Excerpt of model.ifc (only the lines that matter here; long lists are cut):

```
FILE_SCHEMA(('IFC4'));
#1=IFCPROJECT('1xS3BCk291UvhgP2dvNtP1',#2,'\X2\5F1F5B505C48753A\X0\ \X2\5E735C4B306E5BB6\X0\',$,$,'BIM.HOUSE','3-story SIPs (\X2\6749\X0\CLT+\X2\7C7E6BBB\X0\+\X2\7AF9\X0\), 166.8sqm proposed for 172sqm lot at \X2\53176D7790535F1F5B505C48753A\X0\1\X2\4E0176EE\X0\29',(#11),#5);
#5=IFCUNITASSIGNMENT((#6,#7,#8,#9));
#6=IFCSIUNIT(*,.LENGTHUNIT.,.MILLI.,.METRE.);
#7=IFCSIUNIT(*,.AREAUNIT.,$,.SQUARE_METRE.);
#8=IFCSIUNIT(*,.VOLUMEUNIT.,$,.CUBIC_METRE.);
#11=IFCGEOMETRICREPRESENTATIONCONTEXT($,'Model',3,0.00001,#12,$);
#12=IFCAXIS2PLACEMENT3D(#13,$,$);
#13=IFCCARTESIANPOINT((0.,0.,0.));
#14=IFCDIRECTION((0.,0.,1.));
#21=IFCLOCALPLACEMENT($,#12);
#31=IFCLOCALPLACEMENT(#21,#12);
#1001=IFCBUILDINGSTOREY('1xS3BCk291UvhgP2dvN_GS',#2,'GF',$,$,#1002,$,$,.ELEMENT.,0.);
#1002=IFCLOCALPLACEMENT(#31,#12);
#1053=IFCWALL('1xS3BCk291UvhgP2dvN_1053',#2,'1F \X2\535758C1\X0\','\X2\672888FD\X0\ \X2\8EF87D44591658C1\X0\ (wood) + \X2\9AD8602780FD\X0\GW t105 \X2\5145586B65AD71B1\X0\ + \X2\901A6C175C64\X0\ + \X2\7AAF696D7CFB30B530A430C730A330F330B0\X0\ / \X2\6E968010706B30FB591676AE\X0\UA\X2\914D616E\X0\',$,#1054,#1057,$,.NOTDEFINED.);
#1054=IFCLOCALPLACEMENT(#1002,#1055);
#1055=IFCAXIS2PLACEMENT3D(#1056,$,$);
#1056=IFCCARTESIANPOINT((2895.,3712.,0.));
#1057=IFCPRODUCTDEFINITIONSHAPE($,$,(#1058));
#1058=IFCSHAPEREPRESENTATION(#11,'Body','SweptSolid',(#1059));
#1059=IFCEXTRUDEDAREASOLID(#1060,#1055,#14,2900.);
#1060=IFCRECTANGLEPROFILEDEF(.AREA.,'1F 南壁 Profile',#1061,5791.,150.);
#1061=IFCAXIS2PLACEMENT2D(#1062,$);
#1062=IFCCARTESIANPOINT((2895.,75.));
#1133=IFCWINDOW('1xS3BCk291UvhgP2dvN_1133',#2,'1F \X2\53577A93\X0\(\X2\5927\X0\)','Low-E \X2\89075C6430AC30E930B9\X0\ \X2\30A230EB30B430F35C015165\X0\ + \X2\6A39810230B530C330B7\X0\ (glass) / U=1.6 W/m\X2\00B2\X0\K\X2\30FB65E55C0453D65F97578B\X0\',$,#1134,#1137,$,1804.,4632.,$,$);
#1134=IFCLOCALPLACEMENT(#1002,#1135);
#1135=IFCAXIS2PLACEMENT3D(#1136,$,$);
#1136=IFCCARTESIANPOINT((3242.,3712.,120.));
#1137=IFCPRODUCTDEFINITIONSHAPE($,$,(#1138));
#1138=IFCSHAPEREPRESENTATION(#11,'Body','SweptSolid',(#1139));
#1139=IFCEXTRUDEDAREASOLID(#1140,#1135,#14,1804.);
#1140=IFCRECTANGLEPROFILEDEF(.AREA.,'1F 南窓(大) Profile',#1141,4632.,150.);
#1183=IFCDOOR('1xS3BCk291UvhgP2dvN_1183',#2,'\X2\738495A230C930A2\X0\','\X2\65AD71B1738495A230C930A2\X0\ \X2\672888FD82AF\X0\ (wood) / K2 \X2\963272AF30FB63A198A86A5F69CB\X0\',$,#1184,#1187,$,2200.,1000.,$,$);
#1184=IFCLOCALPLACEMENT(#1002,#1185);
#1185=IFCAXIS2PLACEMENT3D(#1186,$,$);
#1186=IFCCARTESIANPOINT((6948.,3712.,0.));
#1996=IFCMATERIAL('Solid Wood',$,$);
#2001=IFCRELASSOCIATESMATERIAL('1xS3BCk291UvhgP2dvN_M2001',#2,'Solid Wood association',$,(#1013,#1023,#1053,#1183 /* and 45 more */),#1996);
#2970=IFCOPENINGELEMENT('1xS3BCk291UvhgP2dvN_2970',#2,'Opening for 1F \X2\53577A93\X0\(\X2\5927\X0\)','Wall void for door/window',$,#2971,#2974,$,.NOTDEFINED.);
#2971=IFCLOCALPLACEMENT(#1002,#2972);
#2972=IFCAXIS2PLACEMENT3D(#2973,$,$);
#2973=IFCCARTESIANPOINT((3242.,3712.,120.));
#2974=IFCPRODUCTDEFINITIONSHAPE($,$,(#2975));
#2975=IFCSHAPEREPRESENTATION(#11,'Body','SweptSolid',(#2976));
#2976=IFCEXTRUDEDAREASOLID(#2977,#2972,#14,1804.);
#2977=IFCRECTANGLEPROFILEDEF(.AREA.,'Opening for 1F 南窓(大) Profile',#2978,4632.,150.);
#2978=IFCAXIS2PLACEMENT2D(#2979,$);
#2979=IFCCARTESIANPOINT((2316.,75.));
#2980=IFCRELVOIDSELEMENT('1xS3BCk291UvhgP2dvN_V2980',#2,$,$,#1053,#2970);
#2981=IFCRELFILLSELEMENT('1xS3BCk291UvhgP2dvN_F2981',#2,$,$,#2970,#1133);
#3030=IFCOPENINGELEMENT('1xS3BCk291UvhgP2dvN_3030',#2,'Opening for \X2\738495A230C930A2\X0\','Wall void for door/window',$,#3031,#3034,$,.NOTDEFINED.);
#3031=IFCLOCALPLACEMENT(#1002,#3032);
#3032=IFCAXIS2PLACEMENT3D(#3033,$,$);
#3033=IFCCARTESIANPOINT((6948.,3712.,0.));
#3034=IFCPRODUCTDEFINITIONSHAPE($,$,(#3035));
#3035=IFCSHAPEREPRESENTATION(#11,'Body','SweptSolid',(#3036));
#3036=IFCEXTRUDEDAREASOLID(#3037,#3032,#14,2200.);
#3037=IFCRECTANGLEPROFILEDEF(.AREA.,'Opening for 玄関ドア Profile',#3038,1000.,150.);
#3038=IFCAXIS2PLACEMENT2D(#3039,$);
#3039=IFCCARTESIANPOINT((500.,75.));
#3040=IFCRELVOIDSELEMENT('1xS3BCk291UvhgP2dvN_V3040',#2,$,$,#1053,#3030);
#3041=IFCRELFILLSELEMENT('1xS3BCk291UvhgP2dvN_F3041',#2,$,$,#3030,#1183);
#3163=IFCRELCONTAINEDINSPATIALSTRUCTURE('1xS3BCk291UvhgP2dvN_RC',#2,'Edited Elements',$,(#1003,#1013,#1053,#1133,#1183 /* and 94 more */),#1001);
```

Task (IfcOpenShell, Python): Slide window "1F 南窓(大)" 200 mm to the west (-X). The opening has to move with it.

```python
import ifcopenshell
import ifcopenshell.api.geometry
import ifcopenshell.util.placement
import ifcopenshell.util.unit

model = ifcopenshell.open("model.ifc")
unit_scale = ifcopenshell.util.unit.calculate_unit_scale(model)

window = model.by_guid("1xS3BCk291UvhgP2dvN_1133")
opening = window.FillsVoids[0].RelatingOpeningElement
wall = opening.VoidsElements[0].RelatingBuildingElement

wall_matrix = ifcopenshell.util.placement.get_local_placement(wall.ObjectPlacement)
shift = wall_matrix[:3, 0] * -0.2 / unit_scale
before = ifcopenshell.util.placement.get_local_placement(window.ObjectPlacement)[:3, 3].copy()

# The window is not placed relative to its opening, so move both.
for product in (opening, window):
    matrix = ifcopenshell.util.placement.get_local_placement(product.ObjectPlacement)
    matrix[:3, 3] += shift
    ifcopenshell.api.geometry.edit_object_placement(model, product=product, matrix=matrix, is_si=False)

after = ifcopenshell.util.placement.get_local_placement(window.ObjectPlacement)[:3, 3]
print("window moved by", (after - before).round(3) + 0.0)

model.write("model_v2.ifc")
```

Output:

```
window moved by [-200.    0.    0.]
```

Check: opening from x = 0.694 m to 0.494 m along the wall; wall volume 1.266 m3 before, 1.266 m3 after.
